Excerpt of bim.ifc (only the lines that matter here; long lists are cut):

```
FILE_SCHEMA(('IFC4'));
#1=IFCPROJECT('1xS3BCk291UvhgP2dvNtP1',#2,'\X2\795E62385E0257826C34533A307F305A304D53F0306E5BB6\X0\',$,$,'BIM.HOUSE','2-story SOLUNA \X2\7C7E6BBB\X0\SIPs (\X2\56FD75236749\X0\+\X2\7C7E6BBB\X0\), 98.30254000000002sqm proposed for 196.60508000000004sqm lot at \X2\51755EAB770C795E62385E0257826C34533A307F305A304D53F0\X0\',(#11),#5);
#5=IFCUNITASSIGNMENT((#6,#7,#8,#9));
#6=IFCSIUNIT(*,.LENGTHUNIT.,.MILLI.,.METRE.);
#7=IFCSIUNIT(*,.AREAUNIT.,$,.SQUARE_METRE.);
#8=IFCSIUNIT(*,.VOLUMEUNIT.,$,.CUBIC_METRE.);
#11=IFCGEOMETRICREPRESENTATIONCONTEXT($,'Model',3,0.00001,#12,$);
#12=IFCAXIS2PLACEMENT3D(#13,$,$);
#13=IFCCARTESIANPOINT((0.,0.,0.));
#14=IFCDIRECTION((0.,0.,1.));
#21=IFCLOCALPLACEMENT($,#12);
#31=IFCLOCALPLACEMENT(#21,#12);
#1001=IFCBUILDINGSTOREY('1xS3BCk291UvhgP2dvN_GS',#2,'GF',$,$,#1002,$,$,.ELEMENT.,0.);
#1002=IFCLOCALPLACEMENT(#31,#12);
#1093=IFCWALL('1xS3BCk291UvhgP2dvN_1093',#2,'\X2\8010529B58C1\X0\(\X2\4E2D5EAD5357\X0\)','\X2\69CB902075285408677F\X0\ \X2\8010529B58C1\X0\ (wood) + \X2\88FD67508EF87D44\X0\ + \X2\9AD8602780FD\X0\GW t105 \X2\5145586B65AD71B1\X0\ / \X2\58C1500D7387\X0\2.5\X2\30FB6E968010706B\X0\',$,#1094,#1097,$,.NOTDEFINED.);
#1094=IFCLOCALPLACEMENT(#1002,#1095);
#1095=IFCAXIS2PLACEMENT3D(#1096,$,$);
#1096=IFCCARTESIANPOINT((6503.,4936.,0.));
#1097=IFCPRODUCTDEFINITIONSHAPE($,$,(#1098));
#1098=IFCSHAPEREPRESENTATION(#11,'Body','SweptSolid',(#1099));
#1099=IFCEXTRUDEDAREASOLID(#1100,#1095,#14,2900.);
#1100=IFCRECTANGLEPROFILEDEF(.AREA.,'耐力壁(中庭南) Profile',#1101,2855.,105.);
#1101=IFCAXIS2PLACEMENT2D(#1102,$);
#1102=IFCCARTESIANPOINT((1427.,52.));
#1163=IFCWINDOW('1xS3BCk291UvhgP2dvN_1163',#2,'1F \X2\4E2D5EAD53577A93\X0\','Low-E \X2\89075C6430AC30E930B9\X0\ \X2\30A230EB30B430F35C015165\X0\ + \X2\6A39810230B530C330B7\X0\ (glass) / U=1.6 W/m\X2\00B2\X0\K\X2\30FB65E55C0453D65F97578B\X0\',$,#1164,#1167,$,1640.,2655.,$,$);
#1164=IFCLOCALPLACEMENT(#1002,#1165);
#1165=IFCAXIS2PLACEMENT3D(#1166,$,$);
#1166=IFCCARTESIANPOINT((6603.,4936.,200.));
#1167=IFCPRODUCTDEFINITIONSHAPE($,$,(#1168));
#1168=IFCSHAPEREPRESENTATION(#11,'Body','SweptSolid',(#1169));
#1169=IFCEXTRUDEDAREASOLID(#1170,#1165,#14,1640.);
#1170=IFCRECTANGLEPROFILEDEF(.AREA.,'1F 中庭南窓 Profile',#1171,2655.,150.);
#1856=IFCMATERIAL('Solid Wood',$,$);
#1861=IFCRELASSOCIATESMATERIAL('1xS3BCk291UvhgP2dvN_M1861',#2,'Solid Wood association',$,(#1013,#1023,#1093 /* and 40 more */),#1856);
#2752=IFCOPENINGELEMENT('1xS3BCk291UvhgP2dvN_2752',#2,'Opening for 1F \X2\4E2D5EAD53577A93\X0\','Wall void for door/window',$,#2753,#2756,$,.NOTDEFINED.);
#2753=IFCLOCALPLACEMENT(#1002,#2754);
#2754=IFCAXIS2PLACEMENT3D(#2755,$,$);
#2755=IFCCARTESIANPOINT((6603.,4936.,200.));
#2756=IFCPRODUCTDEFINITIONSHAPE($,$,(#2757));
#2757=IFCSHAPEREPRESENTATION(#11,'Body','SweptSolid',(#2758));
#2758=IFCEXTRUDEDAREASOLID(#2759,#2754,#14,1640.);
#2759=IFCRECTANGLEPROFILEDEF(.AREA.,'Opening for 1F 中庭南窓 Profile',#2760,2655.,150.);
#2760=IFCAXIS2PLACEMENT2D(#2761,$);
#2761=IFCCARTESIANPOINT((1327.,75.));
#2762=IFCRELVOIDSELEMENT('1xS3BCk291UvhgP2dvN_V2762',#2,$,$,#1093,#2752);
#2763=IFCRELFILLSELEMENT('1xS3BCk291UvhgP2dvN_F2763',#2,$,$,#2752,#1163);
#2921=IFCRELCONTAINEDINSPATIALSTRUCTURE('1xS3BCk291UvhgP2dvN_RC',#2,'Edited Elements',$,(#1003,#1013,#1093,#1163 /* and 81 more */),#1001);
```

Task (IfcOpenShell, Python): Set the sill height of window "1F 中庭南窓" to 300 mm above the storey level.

```python
import numpy as np
import ifcopenshell
import ifcopenshell.api.geometry
import ifcopenshell.geom
import ifcopenshell.util.element
import ifcopenshell.util.placement
import ifcopenshell.util.shape
import ifcopenshell.util.unit

model = ifcopenshell.open("bim.ifc")
unit_scale = ifcopenshell.util.unit.calculate_unit_scale(model)

window = model.by_guid("1xS3BCk291UvhgP2dvN_1163")
opening = window.FillsVoids[0].RelatingOpeningElement
storey = ifcopenshell.util.element.get_container(window, ifc_class="IfcBuildingStorey")
level = ifcopenshell.util.placement.get_local_placement(storey.ObjectPlacement)[2, 3]

# The opening's origin need not be at the sill, so measure its lowest point.
shape = ifcopenshell.geom.create_shape(ifcopenshell.geom.settings(), opening)
bottom = ifcopenshell.util.shape.get_shape_bottom_elevation(shape, shape.geometry) / unit_scale
dz = level + 300.0 - bottom

shift = np.array([0.0, 0.0, dz])
# The window is not placed relative to its opening, so move both.
for product in (opening, window):
    matrix = ifcopenshell.util.placement.get_local_placement(product.ObjectPlacement)
    matrix[:3, 3] += shift
    ifcopenshell.api.geometry.edit_object_placement(model, product=product, matrix=matrix, is_si=False)

print(f"moved by {dz * unit_scale:+.3f} m")

model.write("bim-out.ifc")
```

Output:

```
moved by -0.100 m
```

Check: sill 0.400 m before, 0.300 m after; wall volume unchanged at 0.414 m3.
